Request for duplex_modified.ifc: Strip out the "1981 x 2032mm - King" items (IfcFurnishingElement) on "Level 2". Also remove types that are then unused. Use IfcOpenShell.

First a look at what the model holds.

```python
import ifcopenshell
import ifcopenshell.util.element

model = ifcopenshell.open("duplex_modified.ifc")
print(model.schema)
storey = next(s for s in model.by_type("IfcBuildingStorey") if s.Name == "Level 2")
furniture = [e for e in ifcopenshell.util.element.get_decomposition(storey) if e.is_a("IfcFurnishingElement")]
seen = {}
for e in furniture:
    element_type = ifcopenshell.util.element.get_type(e)
    name = element_type.Name if element_type not in (None, e) else None
    seen[name] = seen.get(name, 0) + 1
for name, count in sorted(seen.items(), key=str):
    print(count, "x", name)
```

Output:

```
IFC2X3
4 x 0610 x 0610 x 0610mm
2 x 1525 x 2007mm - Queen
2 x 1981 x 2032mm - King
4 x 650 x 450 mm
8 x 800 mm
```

```python
import ifcopenshell
import ifcopenshell.api.root
import ifcopenshell.util.element

model = ifcopenshell.open("duplex_modified.ifc")

storey = next(s for s in model.by_type("IfcBuildingStorey") if s.Name == "Level 2")
furniture = [e for e in ifcopenshell.util.element.get_decomposition(storey) if e.is_a("IfcFurnishingElement")]
targets = [e for e in furniture if (t := ifcopenshell.util.element.get_type(e)) not in (None, e) and t.Name == "1981 x 2032mm - King"]
types = {ifcopenshell.util.element.get_type(e) for e in targets} - {None, *targets}

for e in targets:
    ifcopenshell.api.root.remove_product(model, product=e)
print(len(targets), "removed")

unused = [t for t in types if not ifcopenshell.util.element.get_types(t)]
for t in unused:
    ifcopenshell.api.root.remove_product(model, product=t)
print(len(unused), "unused types removed")

model.write("duplex_modified-out.ifc")
```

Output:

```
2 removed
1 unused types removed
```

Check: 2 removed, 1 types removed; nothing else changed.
